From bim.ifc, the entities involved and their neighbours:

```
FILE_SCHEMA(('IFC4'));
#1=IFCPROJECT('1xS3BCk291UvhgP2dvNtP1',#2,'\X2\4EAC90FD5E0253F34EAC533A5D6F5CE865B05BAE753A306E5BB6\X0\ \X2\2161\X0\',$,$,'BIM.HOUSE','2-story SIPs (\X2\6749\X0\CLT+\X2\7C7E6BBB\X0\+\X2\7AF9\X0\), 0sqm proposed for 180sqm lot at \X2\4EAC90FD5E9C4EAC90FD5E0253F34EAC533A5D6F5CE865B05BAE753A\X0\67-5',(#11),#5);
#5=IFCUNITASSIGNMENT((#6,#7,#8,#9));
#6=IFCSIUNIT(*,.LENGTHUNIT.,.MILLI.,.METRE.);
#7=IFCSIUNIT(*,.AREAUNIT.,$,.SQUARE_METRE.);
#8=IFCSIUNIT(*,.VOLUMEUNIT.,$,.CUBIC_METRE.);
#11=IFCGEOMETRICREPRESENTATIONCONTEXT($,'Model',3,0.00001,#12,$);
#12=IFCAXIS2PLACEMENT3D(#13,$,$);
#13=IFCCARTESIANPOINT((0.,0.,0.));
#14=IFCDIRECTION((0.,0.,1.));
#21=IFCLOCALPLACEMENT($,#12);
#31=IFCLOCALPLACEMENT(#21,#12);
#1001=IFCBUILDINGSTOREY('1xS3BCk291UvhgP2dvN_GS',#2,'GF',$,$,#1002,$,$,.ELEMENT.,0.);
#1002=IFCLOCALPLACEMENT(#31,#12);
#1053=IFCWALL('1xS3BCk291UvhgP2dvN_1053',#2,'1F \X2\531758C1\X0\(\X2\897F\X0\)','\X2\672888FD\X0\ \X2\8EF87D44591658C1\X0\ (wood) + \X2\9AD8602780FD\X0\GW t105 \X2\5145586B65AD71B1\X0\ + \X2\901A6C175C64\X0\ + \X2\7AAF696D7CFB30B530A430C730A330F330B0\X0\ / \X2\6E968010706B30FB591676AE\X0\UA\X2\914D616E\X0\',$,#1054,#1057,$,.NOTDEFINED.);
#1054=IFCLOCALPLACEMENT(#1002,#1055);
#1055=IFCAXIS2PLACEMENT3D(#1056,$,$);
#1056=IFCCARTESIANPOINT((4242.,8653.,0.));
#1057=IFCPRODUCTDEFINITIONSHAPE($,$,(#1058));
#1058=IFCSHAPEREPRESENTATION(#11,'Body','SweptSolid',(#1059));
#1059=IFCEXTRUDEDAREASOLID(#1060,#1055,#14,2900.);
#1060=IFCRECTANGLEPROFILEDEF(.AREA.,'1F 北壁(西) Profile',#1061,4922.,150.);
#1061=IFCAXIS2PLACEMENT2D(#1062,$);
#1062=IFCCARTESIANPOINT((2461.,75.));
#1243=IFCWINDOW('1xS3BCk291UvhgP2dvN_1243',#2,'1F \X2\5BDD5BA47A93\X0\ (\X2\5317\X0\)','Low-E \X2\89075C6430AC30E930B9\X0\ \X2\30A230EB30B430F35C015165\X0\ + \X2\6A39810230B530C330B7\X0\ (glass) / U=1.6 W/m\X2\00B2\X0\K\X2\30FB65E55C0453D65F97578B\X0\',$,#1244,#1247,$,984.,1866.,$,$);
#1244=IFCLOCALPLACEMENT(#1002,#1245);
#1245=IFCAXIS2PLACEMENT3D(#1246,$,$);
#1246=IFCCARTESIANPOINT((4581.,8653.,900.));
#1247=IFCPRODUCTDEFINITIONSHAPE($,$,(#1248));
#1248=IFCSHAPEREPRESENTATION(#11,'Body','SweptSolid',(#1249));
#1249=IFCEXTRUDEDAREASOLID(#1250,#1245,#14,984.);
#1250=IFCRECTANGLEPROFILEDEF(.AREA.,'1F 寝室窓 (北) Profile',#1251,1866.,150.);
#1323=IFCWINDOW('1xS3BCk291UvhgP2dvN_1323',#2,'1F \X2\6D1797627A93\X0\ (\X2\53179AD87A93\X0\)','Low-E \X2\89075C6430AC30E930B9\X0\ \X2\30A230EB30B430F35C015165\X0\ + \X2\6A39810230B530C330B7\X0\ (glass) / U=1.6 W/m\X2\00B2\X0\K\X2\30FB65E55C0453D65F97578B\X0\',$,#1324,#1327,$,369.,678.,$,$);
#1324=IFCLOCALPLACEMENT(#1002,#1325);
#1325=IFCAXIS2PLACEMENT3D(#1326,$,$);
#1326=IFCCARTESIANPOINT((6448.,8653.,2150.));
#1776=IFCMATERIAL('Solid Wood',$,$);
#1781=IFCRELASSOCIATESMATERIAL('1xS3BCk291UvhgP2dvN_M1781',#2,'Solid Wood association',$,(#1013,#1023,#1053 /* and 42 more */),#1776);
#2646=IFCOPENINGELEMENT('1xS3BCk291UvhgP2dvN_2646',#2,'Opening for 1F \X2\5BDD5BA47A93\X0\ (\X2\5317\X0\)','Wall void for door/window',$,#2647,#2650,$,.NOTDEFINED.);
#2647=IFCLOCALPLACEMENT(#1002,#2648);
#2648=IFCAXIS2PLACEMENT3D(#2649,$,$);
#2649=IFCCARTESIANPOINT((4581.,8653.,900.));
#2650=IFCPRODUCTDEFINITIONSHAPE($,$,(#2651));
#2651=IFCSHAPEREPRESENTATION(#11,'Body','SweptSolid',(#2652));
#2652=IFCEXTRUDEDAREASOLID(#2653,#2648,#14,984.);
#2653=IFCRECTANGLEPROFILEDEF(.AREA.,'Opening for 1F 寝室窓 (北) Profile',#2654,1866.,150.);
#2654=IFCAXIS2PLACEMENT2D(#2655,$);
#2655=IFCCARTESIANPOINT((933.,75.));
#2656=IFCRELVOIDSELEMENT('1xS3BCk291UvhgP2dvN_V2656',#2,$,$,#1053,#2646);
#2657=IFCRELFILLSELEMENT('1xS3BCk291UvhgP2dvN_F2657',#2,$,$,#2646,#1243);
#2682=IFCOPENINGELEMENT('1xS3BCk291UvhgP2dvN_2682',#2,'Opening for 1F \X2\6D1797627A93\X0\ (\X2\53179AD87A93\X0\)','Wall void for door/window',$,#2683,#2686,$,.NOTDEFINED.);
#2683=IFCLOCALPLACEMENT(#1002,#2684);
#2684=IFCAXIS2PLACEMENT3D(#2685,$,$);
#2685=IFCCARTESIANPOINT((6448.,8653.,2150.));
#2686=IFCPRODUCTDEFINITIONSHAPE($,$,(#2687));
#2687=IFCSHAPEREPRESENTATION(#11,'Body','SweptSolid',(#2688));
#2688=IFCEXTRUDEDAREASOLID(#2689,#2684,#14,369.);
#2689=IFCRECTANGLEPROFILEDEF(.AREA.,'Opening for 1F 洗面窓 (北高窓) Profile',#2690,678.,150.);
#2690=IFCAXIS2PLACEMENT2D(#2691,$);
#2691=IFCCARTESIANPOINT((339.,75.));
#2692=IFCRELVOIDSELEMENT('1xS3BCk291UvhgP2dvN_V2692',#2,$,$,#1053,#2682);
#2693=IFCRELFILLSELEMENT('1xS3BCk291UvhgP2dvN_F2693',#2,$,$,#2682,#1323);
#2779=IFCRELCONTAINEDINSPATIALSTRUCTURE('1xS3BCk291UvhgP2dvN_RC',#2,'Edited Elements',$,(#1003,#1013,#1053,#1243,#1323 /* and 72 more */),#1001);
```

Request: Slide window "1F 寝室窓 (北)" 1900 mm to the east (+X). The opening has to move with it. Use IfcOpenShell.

```python
import ifcopenshell
import ifcopenshell.api.geometry
import ifcopenshell.util.placement

model = ifcopenshell.open("bim.ifc")

window = model.by_guid("1xS3BCk291UvhgP2dvN_1243")
opening = window.FillsVoids[0].RelatingOpeningElement
wall = opening.VoidsElements[0].RelatingBuildingElement

wall_matrix = ifcopenshell.util.placement.get_local_placement(wall.ObjectPlacement)
shift = wall_matrix[:3, 0] * 1900.0
before = ifcopenshell.util.placement.get_local_placement(window.ObjectPlacement)[:3, 3].copy()

# The window is not placed relative to its opening, so move both.
for product in (opening, window):
    matrix = ifcopenshell.util.placement.get_local_placement(product.ObjectPlacement)
    matrix[:3, 3] += shift
    ifcopenshell.api.geometry.edit_object_placement(model, product=product, matrix=matrix, is_si=False)

after = ifcopenshell.util.placement.get_local_placement(window.ObjectPlacement)[:3, 3]
print("window moved by", (after - before).round(3) + 0.0)

model.write("bim_v2.ifc")
```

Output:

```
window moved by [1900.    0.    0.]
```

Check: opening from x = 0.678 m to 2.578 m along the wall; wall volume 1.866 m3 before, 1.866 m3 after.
